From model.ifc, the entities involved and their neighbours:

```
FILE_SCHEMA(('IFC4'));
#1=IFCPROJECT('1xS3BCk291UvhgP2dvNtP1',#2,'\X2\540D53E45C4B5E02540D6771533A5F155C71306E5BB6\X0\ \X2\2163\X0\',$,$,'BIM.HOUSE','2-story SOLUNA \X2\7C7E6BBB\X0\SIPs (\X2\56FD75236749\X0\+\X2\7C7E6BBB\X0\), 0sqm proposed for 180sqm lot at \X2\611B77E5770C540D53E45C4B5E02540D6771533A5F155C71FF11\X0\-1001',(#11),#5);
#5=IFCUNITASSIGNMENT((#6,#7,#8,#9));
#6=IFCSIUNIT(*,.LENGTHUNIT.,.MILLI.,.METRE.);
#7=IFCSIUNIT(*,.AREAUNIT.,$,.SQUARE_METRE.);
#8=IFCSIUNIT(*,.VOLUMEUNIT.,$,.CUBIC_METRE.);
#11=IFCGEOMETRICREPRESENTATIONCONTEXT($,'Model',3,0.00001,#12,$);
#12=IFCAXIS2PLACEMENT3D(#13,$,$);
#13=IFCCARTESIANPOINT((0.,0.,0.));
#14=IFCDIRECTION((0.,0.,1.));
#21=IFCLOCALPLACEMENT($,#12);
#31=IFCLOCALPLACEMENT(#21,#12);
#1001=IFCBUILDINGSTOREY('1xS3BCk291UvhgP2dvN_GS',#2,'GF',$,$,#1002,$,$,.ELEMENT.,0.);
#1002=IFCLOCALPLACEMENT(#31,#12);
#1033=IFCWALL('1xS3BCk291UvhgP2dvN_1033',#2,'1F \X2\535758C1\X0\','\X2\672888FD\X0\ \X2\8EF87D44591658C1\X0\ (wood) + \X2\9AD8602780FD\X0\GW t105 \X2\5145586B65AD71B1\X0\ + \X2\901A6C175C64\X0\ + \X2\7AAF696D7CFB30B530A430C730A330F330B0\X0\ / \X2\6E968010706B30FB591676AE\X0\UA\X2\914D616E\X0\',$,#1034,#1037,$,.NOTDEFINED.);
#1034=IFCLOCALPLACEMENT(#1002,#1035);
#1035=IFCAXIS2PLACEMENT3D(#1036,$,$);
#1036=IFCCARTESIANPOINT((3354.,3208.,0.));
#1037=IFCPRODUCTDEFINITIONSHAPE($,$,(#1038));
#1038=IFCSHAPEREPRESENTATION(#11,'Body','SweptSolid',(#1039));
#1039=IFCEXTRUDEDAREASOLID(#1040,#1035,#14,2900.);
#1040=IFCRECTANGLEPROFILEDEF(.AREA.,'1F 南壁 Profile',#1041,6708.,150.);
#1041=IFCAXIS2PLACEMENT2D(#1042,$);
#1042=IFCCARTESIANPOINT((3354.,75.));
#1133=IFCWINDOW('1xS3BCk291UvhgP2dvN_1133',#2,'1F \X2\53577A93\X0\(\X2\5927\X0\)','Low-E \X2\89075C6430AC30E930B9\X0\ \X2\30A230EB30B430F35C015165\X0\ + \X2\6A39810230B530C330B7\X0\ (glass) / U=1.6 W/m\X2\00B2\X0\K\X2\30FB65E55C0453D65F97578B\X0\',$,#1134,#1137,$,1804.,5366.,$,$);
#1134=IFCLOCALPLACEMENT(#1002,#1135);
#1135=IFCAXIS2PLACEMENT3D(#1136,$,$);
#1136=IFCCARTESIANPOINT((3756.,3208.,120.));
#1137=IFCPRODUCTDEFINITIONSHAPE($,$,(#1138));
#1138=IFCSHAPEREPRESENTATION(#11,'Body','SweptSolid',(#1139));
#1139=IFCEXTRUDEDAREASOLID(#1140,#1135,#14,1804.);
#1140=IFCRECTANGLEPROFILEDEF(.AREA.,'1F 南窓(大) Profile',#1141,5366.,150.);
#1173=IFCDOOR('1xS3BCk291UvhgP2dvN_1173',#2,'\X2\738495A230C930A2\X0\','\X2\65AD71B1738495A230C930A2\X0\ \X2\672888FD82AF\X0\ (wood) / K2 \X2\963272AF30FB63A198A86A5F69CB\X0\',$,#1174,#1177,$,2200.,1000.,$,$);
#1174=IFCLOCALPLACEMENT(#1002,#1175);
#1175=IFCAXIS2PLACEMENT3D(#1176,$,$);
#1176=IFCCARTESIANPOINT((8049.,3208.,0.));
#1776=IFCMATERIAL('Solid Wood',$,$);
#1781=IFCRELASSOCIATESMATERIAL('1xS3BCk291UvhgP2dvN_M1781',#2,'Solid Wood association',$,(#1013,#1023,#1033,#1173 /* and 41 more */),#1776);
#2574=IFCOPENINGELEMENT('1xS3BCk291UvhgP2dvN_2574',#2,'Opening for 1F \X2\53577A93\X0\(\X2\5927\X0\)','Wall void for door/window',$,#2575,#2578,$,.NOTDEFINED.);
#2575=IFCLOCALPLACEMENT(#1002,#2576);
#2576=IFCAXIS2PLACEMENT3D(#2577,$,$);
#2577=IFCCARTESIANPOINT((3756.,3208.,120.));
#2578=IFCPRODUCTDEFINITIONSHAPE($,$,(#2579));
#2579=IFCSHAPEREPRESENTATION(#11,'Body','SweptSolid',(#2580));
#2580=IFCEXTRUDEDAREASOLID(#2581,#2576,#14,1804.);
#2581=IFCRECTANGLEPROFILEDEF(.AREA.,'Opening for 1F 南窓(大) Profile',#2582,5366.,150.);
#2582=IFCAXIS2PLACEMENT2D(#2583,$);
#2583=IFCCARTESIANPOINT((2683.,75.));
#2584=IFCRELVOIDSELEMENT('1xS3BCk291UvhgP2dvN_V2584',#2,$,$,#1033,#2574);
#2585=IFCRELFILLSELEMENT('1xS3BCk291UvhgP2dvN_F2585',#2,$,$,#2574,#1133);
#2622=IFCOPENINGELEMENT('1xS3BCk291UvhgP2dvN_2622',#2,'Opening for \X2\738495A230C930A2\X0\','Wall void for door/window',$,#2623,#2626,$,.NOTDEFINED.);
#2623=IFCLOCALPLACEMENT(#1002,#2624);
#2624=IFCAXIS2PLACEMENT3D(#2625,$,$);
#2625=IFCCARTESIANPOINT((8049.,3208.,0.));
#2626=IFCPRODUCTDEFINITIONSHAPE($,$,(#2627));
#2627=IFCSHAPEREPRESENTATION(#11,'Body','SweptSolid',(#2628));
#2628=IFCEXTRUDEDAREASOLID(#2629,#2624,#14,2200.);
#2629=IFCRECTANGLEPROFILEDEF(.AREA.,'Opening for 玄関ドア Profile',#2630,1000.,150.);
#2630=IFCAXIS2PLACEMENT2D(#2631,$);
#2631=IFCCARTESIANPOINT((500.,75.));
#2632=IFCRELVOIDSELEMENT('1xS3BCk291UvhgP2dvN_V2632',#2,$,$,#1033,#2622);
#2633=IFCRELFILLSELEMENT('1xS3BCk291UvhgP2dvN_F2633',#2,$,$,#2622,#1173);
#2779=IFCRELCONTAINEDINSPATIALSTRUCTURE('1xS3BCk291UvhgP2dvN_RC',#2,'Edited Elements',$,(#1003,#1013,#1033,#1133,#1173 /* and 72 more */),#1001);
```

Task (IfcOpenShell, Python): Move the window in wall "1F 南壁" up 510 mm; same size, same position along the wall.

```python
import numpy as np
import ifcopenshell
import ifcopenshell.api.geometry
import ifcopenshell.util.placement
import ifcopenshell.util.unit

model = ifcopenshell.open("model.ifc")
unit_scale = ifcopenshell.util.unit.calculate_unit_scale(model)

window = model.by_id(1133)
opening = window.FillsVoids[0].RelatingOpeningElement
dz = 0.51 / unit_scale

shift = np.array([0.0, 0.0, dz])
# The window is not placed relative to its opening, so move both.
for product in (opening, window):
    matrix = ifcopenshell.util.placement.get_local_placement(product.ObjectPlacement)
    matrix[:3, 3] += shift
    ifcopenshell.api.geometry.edit_object_placement(model, product=product, matrix=matrix, is_si=False)

print(f"moved by {dz * unit_scale:+.3f} m")

model.write("model_v2.ifc")
```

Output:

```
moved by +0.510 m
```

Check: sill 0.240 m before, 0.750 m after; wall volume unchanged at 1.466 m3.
